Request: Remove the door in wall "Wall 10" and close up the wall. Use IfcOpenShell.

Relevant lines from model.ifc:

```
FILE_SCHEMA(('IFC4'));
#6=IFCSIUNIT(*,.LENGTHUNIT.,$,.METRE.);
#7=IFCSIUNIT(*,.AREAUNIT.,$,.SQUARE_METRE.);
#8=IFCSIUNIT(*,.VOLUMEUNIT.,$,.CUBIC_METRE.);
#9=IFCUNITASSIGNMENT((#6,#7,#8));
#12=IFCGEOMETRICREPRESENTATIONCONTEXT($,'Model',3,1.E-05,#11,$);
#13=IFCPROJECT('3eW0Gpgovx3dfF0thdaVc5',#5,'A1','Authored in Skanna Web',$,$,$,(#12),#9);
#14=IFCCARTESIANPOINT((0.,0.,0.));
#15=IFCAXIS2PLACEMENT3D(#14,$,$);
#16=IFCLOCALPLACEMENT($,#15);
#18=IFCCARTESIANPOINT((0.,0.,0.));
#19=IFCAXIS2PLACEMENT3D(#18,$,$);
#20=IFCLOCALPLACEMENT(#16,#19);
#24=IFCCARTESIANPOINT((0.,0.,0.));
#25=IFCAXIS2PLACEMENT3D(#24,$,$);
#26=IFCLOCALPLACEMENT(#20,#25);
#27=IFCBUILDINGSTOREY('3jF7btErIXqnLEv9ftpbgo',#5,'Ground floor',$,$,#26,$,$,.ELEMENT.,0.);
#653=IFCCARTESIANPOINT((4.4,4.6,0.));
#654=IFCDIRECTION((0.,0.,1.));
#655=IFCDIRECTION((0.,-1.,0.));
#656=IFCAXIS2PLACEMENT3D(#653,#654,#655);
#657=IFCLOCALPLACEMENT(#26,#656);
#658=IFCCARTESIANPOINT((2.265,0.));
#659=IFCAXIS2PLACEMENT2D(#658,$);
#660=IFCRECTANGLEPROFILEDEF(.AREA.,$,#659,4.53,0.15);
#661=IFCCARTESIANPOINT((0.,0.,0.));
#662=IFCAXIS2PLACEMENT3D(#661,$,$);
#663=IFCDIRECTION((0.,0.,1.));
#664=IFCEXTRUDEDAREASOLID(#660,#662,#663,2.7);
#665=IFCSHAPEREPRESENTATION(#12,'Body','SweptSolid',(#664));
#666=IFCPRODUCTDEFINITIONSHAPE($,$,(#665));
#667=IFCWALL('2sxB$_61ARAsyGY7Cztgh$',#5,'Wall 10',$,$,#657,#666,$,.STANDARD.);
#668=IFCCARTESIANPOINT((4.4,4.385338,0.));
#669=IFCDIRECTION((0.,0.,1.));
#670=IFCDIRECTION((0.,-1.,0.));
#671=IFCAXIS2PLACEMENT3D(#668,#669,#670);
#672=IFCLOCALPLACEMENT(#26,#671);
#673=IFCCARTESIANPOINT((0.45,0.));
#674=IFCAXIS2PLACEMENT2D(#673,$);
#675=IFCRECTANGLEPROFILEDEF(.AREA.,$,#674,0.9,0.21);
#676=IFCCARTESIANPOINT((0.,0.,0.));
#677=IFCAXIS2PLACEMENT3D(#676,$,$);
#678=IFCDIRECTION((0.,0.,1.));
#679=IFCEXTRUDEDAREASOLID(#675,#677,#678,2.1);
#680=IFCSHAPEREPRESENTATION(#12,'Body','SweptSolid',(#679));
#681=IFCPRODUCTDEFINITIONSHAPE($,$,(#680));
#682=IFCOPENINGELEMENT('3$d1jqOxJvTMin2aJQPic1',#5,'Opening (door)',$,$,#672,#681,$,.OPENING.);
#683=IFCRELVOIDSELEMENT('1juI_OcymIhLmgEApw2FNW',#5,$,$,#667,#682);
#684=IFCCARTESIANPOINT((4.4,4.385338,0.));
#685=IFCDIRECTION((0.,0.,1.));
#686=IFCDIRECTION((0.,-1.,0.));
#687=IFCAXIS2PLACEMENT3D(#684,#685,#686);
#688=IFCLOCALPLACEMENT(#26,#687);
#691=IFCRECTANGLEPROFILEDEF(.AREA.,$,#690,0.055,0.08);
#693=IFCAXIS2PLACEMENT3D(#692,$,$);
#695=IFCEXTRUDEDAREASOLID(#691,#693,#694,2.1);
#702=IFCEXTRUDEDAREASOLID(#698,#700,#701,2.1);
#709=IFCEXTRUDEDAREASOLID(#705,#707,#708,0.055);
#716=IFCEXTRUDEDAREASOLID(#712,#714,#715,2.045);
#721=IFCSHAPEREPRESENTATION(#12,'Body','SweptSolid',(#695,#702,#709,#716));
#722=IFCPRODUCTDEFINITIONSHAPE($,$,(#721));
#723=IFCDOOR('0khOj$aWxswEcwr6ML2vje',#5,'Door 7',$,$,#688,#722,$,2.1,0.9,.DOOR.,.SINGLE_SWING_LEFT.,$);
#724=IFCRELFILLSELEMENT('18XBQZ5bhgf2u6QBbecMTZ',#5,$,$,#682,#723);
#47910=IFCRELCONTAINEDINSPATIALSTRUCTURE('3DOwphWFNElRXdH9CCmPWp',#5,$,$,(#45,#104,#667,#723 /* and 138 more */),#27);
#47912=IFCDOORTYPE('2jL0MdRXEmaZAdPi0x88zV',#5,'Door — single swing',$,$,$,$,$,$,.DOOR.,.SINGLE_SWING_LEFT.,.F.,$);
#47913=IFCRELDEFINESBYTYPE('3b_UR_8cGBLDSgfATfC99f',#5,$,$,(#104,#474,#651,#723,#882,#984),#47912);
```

```python
import ifcopenshell
import ifcopenshell.api.feature
import ifcopenshell.api.root
import ifcopenshell.geom
import ifcopenshell.util.shape

model = ifcopenshell.open("model.ifc")
settings = ifcopenshell.geom.settings()


def volume(element):
    """Net volume in cubic metres, openings subtracted."""
    shape = ifcopenshell.geom.create_shape(settings, element)
    return ifcopenshell.util.shape.get_volume(shape.geometry)


door = model.by_id(723)
opening = door.FillsVoids[0].RelatingOpeningElement
wall = opening.VoidsElements[0].RelatingBuildingElement
before = volume(wall)

ifcopenshell.api.root.remove_product(model, product=door)
ifcopenshell.api.feature.remove_feature(model, feature=opening)

after = volume(wall)

print(f"wall volume {before:.3f} -> {after:.3f} m3")

model.write("model_v2.ifc")
```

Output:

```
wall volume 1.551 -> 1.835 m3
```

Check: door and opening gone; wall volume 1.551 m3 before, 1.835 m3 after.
